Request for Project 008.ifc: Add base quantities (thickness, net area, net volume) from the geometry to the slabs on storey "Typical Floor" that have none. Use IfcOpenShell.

First a look at what the model holds.

```python
import ifcopenshell
import ifcopenshell.util.element
import ifcopenshell.util.unit

model = ifcopenshell.open("Project 008.ifc")
print(model.schema)
for unit_type in ("LENGTHUNIT", "AREAUNIT", "VOLUMEUNIT"):
    print(unit_type, ifcopenshell.util.unit.calculate_unit_scale(model, unit_type))
storey = next(s for s in model.by_type("IfcBuildingStorey") if s.Name == "Typical Floor")
slabs = [e for e in ifcopenshell.util.element.get_decomposition(storey) if e.is_a("IfcSlab")]
for e in sorted(slabs, key=lambda e: e.id()):
    print(e.id(), e.is_a(), e.Name, list(ifcopenshell.util.element.get_psets(e, qtos_only=True)), sep=" | ")
```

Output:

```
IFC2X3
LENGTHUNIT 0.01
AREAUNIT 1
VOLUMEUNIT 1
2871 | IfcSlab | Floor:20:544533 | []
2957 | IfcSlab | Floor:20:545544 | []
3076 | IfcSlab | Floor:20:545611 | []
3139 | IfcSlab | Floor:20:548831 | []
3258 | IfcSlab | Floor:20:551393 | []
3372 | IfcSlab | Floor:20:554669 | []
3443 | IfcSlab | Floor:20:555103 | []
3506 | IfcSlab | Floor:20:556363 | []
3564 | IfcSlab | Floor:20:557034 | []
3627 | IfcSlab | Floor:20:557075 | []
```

```python
import ifcopenshell
import ifcopenshell.api.pset
import ifcopenshell.geom
import ifcopenshell.util.element
import ifcopenshell.util.shape
import ifcopenshell.util.unit

model = ifcopenshell.open("Project 008.ifc")
unit_scale = ifcopenshell.util.unit.calculate_unit_scale(model)
area_scale = ifcopenshell.util.unit.calculate_unit_scale(model, "AREAUNIT")
volume_scale = ifcopenshell.util.unit.calculate_unit_scale(model, "VOLUMEUNIT")
settings = ifcopenshell.geom.settings()

storey = next(s for s in model.by_type("IfcBuildingStorey") if s.Name == "Typical Floor")
slabs = [e for e in ifcopenshell.util.element.get_decomposition(storey) if e.is_a("IfcSlab")]

for e in sorted(slabs, key=lambda e: e.id()):
    if ifcopenshell.util.element.get_psets(e, qtos_only=True, should_inherit=False):
        continue
    # Geometry comes back in metres, in the element's own axes.
    shape = ifcopenshell.geom.create_shape(settings, e)
    values = {
        "Width": ifcopenshell.util.shape.get_z(shape.geometry) / unit_scale,
        "NetArea": ifcopenshell.util.shape.get_footprint_area(shape.geometry) / area_scale,
        "NetVolume": ifcopenshell.util.shape.get_volume(shape.geometry) / volume_scale,
    }
    qto = ifcopenshell.api.pset.add_qto(model, product=e, name="BaseQuantities")
    ifcopenshell.api.pset.edit_qto(model, qto=qto, properties=values)
    print(e.id(), {k: round(v, 3) for k, v in values.items()})

model.write("Project 008-out.ifc")
```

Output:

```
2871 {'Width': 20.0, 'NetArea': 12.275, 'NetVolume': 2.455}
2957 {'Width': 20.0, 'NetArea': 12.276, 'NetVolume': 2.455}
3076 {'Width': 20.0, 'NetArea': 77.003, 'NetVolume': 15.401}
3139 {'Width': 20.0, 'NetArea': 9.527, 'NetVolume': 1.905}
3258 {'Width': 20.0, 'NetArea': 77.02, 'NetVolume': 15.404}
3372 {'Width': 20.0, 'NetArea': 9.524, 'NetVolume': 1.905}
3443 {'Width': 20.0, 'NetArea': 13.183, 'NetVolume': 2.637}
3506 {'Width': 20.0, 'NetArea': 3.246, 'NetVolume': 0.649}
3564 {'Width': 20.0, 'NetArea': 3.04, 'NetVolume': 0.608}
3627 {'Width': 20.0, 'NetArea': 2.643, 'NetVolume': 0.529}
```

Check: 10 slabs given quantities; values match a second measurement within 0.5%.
